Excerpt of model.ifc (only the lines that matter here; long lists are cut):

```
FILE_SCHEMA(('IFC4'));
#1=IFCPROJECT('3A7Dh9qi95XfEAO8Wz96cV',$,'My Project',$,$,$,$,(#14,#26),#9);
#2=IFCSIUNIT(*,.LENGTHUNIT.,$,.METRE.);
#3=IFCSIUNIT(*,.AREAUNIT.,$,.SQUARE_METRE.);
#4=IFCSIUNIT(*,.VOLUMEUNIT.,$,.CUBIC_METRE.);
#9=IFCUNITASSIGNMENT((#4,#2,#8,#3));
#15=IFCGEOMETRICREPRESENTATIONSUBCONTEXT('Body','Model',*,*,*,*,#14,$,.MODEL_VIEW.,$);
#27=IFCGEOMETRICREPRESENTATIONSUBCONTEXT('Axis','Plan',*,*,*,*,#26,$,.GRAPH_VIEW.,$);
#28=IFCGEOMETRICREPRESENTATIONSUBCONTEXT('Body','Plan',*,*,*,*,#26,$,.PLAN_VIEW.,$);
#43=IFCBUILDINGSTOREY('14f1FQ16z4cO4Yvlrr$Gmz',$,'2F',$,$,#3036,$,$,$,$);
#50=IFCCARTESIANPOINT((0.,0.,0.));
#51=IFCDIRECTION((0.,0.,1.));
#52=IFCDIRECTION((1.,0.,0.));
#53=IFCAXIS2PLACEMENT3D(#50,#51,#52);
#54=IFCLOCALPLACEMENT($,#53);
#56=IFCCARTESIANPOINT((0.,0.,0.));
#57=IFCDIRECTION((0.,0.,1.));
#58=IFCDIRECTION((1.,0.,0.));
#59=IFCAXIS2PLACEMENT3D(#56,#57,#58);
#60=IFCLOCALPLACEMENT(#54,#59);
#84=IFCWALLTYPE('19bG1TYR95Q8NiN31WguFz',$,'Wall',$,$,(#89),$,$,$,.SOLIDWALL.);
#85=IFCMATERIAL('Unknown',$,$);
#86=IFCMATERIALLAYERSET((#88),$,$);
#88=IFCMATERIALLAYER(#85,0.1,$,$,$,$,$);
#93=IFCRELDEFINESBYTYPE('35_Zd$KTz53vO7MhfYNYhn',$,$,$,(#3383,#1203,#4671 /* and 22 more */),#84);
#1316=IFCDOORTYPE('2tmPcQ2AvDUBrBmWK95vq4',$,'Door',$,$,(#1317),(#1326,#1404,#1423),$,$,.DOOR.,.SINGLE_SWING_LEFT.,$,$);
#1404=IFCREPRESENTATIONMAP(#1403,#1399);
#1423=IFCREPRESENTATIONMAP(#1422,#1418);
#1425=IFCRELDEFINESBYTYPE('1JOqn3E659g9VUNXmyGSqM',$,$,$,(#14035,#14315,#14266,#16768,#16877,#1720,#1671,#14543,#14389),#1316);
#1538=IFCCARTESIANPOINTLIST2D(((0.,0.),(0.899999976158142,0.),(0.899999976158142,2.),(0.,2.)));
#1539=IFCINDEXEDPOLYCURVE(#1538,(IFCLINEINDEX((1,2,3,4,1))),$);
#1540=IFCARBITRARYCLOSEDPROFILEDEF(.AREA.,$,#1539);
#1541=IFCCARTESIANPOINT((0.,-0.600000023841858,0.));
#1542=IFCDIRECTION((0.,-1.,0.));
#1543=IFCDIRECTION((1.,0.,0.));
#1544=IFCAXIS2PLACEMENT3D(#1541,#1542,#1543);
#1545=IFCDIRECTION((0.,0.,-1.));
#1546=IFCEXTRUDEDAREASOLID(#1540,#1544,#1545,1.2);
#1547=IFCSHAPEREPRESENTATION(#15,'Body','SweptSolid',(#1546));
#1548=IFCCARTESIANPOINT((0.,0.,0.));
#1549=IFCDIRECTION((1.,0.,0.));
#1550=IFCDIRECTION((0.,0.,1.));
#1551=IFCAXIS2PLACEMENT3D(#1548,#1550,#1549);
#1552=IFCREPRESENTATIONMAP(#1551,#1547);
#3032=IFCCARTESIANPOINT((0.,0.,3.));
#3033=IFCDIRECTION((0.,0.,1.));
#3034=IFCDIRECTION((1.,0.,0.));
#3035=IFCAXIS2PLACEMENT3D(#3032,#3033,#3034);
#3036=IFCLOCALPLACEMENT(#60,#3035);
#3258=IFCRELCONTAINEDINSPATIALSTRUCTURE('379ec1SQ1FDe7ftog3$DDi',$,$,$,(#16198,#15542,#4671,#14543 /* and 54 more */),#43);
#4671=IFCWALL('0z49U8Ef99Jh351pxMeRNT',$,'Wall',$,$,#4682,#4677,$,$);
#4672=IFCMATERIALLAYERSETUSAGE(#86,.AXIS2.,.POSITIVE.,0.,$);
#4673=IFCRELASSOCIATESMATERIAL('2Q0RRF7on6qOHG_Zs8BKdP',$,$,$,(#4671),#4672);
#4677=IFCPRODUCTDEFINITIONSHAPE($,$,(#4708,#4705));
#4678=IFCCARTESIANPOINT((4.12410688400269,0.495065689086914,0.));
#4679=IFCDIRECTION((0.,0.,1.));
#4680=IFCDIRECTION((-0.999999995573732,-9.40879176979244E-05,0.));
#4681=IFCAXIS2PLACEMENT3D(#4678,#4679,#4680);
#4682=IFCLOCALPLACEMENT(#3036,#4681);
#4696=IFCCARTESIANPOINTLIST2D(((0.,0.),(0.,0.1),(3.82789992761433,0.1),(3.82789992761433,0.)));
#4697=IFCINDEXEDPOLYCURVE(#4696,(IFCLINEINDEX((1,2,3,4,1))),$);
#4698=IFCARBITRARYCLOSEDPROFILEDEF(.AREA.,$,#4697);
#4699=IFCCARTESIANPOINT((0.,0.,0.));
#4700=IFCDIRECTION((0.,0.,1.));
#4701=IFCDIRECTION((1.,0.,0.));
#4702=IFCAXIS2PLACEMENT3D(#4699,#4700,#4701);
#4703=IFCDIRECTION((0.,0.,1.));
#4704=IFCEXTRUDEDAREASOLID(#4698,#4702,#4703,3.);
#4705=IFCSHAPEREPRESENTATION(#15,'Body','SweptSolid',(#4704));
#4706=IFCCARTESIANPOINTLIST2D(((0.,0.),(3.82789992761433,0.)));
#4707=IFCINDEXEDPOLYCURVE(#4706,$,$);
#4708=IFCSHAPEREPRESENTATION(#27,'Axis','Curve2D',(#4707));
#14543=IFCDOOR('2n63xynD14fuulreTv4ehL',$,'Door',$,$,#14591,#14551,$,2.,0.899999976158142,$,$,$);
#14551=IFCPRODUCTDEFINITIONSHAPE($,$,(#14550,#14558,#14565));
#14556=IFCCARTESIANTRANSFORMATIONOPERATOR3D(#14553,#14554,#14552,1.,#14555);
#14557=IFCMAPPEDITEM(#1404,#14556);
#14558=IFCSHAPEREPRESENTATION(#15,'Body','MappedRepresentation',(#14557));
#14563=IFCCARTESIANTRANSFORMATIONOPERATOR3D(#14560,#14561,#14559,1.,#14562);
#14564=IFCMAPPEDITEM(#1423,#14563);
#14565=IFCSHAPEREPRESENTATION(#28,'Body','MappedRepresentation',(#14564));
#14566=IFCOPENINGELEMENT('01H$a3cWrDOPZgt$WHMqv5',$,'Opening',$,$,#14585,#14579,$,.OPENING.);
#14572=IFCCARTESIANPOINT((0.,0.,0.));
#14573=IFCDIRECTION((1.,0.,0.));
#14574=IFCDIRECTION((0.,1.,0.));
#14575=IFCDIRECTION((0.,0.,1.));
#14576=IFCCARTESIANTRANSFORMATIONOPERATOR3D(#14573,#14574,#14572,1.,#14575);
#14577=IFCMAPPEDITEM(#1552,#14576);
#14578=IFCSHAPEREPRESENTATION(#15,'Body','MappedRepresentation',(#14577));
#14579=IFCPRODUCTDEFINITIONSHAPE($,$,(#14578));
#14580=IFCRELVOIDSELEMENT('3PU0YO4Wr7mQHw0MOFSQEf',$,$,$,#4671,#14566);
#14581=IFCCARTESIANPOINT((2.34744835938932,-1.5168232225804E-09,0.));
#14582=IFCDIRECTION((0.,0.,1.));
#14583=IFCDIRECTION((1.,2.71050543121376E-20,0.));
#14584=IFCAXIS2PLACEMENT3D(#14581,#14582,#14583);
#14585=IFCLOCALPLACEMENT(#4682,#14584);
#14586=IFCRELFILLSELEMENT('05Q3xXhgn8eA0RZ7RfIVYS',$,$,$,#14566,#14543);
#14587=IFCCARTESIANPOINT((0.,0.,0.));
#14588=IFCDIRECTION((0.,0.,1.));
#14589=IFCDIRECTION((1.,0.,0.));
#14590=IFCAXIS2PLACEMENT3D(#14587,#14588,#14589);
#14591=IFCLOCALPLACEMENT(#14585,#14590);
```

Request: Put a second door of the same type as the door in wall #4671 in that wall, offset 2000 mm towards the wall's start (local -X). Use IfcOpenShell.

```python
import ifcopenshell
import ifcopenshell.api.feature
import ifcopenshell.api.geometry
import ifcopenshell.api.root
import ifcopenshell.geom
import ifcopenshell.util.element
import ifcopenshell.util.placement
import ifcopenshell.util.shape

model = ifcopenshell.open("model.ifc")
settings = ifcopenshell.geom.settings()


def volume(element):
    """Net volume in cubic metres, openings subtracted."""
    shape = ifcopenshell.geom.create_shape(settings, element)
    return ifcopenshell.util.shape.get_volume(shape.geometry)


door = model.by_id(14543)
opening = door.FillsVoids[0].RelatingOpeningElement
wall = opening.VoidsElements[0].RelatingBuildingElement
before = volume(wall)
shift = ifcopenshell.util.placement.get_local_placement(wall.ObjectPlacement)[:3, 0] * -2.0

# copy_class copies the void relationship, type, container and properties, but no geometry.
new_opening = ifcopenshell.api.root.copy_class(model, product=opening)
new_opening.Representation = ifcopenshell.util.element.copy_deep(
    model, opening.Representation, exclude=["IfcGeometricRepresentationContext", "IfcRepresentationMap"]
)
new_door = ifcopenshell.api.root.copy_class(model, product=door)
new_door.Representation = ifcopenshell.util.element.copy_deep(
    model, door.Representation, exclude=["IfcGeometricRepresentationContext", "IfcRepresentationMap"]
)
ifcopenshell.api.feature.add_filling(model, opening=new_opening, element=new_door)

for old, new in ((opening, new_opening), (door, new_door)):
    matrix = ifcopenshell.util.placement.get_local_placement(old.ObjectPlacement)
    matrix[:3, 3] += shift
    ifcopenshell.api.geometry.edit_object_placement(model, product=new, matrix=matrix, is_si=False)

after = volume(wall)

print(f"wall volume {before:.3f} -> {after:.3f} m3")

model.write("model-out.ifc")
```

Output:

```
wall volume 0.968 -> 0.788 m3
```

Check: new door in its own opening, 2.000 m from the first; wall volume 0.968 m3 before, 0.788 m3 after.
